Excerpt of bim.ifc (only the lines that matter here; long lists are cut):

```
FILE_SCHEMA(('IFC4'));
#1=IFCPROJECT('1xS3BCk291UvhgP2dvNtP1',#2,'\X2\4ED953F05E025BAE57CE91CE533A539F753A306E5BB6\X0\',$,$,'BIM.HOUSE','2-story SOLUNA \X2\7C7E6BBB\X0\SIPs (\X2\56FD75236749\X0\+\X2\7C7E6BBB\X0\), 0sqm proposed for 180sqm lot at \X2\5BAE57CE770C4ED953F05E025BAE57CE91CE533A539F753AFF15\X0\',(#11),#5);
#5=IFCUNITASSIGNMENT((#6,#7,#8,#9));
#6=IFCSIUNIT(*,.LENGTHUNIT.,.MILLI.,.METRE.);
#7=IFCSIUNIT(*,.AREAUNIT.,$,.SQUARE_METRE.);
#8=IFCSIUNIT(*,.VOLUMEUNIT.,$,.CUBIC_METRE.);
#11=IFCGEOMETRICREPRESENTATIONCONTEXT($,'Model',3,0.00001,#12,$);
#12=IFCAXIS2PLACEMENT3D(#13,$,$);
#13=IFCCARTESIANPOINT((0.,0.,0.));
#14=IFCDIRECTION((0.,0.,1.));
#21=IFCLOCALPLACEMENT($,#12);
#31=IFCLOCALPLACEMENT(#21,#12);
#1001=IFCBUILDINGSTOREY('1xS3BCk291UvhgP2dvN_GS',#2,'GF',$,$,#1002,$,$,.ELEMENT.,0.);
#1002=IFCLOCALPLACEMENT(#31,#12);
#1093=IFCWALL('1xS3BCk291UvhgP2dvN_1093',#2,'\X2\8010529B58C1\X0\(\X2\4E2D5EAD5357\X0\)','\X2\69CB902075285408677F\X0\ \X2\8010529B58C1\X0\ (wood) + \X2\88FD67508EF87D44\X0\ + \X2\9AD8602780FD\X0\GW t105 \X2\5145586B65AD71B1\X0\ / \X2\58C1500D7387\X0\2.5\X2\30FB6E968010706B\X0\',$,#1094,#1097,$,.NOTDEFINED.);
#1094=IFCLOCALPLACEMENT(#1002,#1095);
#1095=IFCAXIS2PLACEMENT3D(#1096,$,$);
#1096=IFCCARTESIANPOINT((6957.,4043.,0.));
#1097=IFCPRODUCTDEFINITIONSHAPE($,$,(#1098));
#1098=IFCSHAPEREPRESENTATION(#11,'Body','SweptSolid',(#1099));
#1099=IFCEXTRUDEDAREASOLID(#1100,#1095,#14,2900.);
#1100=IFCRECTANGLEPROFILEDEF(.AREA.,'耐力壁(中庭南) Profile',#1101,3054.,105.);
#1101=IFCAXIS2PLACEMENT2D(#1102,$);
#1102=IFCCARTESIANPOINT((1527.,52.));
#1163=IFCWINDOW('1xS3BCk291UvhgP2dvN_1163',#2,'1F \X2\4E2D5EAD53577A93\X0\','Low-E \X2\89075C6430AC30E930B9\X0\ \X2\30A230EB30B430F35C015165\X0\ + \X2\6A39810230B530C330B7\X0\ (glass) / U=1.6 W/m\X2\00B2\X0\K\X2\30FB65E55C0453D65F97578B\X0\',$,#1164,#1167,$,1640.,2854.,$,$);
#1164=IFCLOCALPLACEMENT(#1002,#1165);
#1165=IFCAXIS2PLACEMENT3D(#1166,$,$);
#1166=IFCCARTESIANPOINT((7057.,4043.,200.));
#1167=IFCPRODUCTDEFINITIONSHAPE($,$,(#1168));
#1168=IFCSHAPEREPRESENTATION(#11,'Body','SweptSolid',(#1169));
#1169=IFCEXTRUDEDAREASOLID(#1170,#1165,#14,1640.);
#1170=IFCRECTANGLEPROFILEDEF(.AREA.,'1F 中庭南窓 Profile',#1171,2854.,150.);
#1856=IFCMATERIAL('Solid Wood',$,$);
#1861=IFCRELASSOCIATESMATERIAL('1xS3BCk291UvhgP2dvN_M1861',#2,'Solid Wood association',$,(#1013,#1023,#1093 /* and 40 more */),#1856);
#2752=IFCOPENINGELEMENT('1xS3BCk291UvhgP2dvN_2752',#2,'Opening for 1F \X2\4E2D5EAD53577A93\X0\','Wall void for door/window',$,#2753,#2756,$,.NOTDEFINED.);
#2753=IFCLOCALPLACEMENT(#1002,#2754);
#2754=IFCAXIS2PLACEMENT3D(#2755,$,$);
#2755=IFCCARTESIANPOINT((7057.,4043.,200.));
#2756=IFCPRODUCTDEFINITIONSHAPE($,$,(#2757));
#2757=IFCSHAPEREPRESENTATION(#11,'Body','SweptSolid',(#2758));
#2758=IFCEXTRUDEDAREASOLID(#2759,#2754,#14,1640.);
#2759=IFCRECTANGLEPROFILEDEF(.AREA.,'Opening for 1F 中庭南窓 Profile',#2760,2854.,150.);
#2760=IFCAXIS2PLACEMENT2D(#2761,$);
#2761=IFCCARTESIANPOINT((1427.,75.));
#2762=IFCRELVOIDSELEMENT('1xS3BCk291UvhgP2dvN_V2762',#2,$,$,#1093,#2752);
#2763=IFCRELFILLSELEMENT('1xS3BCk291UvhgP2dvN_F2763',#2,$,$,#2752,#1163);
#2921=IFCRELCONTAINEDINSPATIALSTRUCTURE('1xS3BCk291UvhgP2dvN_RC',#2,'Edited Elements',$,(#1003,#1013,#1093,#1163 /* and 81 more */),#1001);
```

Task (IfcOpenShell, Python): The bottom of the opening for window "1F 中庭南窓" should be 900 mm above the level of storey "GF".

```python
import numpy as np
import ifcopenshell
import ifcopenshell.api.geometry
import ifcopenshell.geom
import ifcopenshell.util.element
import ifcopenshell.util.placement
import ifcopenshell.util.shape
import ifcopenshell.util.unit

model = ifcopenshell.open("bim.ifc")
unit_scale = ifcopenshell.util.unit.calculate_unit_scale(model)

window = model.by_id(1163)
opening = window.FillsVoids[0].RelatingOpeningElement
storey = ifcopenshell.util.element.get_container(window, ifc_class="IfcBuildingStorey")
level = ifcopenshell.util.placement.get_local_placement(storey.ObjectPlacement)[2, 3]

# The opening's origin need not be at the sill, so measure its lowest point.
shape = ifcopenshell.geom.create_shape(ifcopenshell.geom.settings(), opening)
bottom = ifcopenshell.util.shape.get_shape_bottom_elevation(shape, shape.geometry) / unit_scale
dz = level + 900.0 - bottom

shift = np.array([0.0, 0.0, dz])
# The window is not placed relative to its opening, so move both.
for product in (opening, window):
    matrix = ifcopenshell.util.placement.get_local_placement(product.ObjectPlacement)
    matrix[:3, 3] += shift
    ifcopenshell.api.geometry.edit_object_placement(model, product=product, matrix=matrix, is_si=False)

print(f"moved by {dz * unit_scale:+.3f} m")

model.write("bim-out.ifc")
```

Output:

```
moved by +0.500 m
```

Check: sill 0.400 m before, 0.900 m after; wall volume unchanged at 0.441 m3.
